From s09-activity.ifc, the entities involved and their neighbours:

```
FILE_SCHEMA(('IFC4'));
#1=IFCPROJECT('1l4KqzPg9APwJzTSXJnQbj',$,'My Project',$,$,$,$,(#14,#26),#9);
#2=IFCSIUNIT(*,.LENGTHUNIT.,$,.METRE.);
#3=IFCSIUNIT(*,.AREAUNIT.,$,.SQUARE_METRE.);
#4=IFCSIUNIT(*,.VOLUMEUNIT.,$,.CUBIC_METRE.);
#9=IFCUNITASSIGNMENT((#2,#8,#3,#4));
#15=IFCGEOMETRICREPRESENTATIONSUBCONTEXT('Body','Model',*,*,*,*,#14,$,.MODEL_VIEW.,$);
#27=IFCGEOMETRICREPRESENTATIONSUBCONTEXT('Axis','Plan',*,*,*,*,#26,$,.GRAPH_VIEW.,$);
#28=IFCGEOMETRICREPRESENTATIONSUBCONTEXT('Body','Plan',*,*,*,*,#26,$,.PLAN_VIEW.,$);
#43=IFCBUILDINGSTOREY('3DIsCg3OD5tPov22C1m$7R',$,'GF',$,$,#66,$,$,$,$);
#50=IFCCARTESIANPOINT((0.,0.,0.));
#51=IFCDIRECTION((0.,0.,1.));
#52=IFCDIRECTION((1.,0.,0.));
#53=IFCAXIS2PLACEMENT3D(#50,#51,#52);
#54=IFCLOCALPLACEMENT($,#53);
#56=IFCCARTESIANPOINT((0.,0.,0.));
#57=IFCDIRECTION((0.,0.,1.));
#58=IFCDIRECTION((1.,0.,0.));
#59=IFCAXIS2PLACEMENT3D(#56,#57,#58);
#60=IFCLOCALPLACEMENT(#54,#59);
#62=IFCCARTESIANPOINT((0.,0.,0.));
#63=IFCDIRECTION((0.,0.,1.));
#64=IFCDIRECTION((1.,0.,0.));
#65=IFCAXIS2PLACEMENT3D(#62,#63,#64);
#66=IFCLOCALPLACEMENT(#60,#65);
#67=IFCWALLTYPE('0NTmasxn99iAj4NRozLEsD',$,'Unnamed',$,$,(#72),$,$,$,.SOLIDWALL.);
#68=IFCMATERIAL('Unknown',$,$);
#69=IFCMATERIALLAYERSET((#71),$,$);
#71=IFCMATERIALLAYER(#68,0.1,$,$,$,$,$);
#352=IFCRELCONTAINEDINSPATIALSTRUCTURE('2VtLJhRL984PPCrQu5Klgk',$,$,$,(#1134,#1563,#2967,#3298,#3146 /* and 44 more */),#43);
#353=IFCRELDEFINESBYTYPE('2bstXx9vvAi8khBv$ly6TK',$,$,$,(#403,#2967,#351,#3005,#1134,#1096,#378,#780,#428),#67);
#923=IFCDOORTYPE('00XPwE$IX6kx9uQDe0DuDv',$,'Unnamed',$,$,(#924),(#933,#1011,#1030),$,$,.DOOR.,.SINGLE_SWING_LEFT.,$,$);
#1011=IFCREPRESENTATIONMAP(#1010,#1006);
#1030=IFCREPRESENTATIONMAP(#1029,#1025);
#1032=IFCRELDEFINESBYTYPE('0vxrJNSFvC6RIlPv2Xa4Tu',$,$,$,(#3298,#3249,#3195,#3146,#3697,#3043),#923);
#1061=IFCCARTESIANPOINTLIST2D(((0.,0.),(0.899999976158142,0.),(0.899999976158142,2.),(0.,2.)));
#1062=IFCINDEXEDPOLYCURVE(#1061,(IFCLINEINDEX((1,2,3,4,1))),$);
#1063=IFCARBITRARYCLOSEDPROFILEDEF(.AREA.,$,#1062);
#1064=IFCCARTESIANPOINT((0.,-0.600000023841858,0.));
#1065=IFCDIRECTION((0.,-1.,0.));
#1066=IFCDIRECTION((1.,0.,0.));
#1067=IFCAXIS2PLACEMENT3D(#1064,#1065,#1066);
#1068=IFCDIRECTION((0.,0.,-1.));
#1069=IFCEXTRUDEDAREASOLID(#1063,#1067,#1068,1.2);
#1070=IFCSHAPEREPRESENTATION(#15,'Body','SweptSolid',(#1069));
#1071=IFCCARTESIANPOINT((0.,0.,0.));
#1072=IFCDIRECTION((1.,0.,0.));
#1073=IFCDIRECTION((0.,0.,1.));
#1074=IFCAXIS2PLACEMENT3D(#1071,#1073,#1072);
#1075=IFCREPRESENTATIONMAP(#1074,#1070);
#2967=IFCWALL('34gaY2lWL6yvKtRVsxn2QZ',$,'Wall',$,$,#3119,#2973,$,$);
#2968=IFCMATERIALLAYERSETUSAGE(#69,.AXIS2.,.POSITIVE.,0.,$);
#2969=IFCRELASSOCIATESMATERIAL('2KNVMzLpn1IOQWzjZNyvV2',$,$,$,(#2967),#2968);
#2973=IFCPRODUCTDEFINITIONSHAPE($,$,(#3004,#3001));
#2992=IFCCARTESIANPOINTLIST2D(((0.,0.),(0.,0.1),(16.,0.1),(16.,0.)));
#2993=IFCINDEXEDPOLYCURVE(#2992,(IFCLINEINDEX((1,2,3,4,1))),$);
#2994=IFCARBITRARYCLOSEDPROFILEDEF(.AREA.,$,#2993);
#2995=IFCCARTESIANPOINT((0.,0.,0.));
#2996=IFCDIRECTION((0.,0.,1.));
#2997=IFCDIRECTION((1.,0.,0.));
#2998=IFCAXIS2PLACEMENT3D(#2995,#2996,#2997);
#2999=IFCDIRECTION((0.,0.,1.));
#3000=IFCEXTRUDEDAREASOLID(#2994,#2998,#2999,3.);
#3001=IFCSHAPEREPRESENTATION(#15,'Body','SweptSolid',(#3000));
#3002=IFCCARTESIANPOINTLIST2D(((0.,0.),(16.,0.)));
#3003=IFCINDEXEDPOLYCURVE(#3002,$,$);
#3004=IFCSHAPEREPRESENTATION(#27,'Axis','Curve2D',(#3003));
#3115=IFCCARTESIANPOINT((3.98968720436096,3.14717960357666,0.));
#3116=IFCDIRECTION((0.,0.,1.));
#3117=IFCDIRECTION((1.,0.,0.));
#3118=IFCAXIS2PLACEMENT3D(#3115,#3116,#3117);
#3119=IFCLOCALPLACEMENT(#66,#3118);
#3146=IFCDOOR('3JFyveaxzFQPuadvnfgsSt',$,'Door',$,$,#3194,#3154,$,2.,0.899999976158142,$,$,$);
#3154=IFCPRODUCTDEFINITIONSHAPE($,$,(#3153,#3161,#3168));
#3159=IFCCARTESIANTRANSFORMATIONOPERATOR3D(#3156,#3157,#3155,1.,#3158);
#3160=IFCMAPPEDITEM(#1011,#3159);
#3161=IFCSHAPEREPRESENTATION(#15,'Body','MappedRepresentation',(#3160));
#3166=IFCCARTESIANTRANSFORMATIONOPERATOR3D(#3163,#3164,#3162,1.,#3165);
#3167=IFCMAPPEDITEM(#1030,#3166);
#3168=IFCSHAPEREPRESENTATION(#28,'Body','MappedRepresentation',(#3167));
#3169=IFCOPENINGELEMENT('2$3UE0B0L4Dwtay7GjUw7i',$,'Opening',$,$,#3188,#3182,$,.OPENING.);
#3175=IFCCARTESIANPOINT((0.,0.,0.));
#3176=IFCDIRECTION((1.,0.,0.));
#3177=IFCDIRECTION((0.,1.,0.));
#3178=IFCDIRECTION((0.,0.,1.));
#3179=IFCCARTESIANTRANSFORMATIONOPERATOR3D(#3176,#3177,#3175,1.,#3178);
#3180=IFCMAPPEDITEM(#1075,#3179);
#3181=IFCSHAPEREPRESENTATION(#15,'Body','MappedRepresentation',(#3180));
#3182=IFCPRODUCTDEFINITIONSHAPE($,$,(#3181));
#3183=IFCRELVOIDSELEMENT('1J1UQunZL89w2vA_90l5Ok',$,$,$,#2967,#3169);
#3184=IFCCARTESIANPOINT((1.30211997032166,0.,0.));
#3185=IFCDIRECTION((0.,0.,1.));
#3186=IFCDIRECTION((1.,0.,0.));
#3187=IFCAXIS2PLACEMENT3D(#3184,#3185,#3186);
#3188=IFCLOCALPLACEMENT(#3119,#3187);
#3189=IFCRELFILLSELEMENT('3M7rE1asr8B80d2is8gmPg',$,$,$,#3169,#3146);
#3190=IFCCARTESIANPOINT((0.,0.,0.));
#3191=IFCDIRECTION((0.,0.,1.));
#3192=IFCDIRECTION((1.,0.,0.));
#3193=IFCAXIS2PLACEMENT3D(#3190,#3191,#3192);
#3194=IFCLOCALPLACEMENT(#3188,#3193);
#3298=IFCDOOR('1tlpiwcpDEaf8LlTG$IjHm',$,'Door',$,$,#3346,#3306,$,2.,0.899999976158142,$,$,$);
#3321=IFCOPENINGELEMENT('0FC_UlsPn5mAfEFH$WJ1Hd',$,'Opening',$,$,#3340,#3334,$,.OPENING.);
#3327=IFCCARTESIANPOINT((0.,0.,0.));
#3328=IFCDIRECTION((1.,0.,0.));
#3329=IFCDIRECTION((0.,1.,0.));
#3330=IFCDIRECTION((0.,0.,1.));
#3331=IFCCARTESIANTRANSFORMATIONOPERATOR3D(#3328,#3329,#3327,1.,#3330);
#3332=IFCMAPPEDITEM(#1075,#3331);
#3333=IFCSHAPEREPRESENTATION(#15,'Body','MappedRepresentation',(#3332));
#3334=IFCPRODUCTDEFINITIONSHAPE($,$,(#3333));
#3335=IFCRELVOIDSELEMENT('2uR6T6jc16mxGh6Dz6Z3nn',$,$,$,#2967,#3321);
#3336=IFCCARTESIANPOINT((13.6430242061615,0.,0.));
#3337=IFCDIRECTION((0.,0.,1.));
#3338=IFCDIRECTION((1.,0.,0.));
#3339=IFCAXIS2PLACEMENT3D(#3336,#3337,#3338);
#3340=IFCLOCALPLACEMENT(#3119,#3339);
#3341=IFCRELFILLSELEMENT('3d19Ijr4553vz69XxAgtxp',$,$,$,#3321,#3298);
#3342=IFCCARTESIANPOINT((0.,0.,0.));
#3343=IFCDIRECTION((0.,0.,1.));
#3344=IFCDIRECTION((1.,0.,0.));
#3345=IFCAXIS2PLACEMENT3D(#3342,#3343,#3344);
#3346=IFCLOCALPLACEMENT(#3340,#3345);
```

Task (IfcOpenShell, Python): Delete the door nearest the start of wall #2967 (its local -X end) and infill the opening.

```python
import ifcopenshell
import ifcopenshell.api.feature
import ifcopenshell.api.root
import ifcopenshell.geom
import ifcopenshell.util.shape

model = ifcopenshell.open("s09-activity.ifc")
settings = ifcopenshell.geom.settings()


def volume(element):
    """Net volume in cubic metres, openings subtracted."""
    shape = ifcopenshell.geom.create_shape(settings, element)
    return ifcopenshell.util.shape.get_volume(shape.geometry)


door = model.by_guid("3JFyveaxzFQPuadvnfgsSt")
opening = door.FillsVoids[0].RelatingOpeningElement
wall = opening.VoidsElements[0].RelatingBuildingElement
before = volume(wall)

ifcopenshell.api.root.remove_product(model, product=door)
ifcopenshell.api.feature.remove_feature(model, feature=opening)

after = volume(wall)

print(f"wall volume {before:.3f} -> {after:.3f} m3")

model.write("s09-activity-out.ifc")
```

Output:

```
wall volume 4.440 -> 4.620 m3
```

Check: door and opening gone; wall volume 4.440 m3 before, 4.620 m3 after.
